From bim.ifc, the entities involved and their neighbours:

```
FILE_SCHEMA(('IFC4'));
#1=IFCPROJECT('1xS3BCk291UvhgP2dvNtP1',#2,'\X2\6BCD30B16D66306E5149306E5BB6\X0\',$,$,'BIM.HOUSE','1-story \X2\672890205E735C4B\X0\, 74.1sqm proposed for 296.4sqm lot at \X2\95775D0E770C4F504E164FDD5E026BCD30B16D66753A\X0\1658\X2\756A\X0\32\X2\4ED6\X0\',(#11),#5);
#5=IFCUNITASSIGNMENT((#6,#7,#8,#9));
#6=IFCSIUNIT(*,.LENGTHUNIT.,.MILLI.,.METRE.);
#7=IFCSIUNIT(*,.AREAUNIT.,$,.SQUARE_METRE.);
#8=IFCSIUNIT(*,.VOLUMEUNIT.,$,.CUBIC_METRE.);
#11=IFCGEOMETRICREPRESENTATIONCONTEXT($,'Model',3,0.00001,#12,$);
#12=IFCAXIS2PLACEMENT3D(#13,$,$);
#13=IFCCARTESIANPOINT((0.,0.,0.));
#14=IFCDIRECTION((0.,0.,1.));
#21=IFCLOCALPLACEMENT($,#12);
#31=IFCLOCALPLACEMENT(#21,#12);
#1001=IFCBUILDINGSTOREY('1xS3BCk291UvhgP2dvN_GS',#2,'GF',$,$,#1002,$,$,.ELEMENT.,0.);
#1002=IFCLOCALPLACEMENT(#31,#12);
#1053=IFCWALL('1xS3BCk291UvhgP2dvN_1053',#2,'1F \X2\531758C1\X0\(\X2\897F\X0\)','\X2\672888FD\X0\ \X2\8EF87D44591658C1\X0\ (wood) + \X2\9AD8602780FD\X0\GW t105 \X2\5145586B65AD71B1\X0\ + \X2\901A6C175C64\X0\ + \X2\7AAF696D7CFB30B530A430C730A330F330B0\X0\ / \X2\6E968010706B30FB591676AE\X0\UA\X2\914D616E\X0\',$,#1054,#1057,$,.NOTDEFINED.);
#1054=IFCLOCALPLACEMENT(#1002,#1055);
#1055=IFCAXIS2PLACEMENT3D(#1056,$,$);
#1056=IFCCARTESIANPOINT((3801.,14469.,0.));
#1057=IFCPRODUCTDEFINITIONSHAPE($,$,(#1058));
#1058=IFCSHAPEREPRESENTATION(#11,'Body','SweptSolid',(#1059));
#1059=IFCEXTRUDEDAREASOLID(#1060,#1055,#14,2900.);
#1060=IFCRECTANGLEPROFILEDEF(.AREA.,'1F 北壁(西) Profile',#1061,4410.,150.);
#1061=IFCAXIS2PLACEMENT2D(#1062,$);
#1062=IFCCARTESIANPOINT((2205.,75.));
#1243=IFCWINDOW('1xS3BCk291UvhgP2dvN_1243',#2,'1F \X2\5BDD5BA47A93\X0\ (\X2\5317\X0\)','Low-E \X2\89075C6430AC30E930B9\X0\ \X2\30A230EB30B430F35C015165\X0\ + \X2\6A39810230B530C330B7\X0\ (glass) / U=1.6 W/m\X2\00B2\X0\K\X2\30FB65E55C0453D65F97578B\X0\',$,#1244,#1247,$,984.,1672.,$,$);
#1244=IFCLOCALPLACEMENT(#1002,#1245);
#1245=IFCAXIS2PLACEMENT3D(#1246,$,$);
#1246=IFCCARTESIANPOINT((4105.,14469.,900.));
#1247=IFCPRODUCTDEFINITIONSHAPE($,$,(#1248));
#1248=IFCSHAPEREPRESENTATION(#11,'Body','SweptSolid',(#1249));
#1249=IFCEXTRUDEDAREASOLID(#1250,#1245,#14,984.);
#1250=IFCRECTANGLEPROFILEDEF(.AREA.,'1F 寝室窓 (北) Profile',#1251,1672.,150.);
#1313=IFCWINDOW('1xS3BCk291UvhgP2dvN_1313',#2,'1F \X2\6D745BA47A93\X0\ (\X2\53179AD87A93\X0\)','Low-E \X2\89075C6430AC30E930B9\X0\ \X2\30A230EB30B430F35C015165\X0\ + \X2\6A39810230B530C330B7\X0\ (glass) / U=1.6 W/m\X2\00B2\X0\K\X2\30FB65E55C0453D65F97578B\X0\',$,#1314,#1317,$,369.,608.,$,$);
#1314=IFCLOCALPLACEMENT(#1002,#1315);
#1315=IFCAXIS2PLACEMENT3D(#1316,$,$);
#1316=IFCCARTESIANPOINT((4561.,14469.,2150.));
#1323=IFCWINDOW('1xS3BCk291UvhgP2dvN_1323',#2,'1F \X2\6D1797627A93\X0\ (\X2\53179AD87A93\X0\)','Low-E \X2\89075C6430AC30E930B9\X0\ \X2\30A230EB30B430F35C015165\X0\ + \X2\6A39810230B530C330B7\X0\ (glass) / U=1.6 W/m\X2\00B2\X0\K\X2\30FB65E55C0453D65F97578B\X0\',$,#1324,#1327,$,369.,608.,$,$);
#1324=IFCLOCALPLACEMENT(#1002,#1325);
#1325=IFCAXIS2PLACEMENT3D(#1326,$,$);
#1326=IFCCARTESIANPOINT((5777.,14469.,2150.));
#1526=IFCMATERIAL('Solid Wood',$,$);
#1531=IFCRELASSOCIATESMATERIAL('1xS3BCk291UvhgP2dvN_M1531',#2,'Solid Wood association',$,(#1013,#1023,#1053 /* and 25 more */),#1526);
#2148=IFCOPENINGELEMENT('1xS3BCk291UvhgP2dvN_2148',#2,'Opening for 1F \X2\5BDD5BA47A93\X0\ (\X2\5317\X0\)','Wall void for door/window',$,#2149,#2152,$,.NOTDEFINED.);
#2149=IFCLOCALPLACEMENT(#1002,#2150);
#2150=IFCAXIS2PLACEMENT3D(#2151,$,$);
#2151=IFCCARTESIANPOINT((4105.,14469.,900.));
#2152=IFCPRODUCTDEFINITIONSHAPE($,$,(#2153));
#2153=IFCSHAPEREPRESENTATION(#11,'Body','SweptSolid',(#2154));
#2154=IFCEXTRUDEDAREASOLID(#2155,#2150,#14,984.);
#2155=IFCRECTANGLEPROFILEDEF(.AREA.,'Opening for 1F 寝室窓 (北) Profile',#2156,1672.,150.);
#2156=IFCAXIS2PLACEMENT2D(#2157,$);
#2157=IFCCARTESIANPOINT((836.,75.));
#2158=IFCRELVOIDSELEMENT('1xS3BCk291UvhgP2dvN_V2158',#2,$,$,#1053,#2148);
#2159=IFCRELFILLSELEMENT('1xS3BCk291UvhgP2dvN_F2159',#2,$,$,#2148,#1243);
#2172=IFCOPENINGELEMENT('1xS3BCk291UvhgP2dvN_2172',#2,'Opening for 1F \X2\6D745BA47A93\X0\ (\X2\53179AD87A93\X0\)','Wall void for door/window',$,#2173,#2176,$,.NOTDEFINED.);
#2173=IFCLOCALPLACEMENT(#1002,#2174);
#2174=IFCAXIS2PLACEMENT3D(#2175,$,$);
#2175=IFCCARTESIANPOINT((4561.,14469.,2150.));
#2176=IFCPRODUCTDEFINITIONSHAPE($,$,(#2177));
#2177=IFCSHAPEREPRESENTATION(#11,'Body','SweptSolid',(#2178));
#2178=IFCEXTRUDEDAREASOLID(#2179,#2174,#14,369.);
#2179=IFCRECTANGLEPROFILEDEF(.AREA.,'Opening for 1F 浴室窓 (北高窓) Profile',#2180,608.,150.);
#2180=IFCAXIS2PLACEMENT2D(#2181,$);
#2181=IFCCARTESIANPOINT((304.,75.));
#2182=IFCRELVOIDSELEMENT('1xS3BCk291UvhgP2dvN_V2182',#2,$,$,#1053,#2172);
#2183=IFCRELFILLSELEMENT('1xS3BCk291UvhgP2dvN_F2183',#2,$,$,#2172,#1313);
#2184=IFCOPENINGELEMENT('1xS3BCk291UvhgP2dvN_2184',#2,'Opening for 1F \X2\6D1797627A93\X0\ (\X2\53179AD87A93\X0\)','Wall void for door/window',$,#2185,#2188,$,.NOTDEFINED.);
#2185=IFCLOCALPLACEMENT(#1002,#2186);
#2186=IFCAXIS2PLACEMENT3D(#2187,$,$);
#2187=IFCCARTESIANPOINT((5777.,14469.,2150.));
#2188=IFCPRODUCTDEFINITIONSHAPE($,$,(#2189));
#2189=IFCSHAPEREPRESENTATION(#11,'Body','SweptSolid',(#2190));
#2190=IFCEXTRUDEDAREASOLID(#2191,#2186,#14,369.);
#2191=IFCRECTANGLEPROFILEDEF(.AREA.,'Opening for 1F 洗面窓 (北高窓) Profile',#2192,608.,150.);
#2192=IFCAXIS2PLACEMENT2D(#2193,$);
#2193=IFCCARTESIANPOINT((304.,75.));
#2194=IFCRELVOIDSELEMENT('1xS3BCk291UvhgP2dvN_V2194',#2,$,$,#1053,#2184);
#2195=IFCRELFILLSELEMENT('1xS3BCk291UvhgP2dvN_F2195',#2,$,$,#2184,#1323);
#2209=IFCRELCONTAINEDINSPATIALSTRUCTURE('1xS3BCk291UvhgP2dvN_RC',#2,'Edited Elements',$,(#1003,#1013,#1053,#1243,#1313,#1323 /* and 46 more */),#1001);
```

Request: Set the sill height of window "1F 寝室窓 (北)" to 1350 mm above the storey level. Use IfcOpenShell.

```python
import numpy as np
import ifcopenshell
import ifcopenshell.api.geometry
import ifcopenshell.geom
import ifcopenshell.util.element
import ifcopenshell.util.placement
import ifcopenshell.util.shape
import ifcopenshell.util.unit

model = ifcopenshell.open("bim.ifc")
unit_scale = ifcopenshell.util.unit.calculate_unit_scale(model)

window = model.by_guid("1xS3BCk291UvhgP2dvN_1243")
opening = window.FillsVoids[0].RelatingOpeningElement
storey = ifcopenshell.util.element.get_container(window, ifc_class="IfcBuildingStorey")
level = ifcopenshell.util.placement.get_local_placement(storey.ObjectPlacement)[2, 3]

# The opening's origin need not be at the sill, so measure its lowest point.
shape = ifcopenshell.geom.create_shape(ifcopenshell.geom.settings(), opening)
bottom = ifcopenshell.util.shape.get_shape_bottom_elevation(shape, shape.geometry) / unit_scale
dz = level + 1.35 / unit_scale - bottom

shift = np.array([0.0, 0.0, dz])
# The window is not placed relative to its opening, so move both.
for product in (opening, window):
    matrix = ifcopenshell.util.placement.get_local_placement(product.ObjectPlacement)
    matrix[:3, 3] += shift
    ifcopenshell.api.geometry.edit_object_placement(model, product=product, matrix=matrix, is_si=False)

print(f"moved by {dz * unit_scale:+.3f} m")

model.write("bim-out.ifc")
```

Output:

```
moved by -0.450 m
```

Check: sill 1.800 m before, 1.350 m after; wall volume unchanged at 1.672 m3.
